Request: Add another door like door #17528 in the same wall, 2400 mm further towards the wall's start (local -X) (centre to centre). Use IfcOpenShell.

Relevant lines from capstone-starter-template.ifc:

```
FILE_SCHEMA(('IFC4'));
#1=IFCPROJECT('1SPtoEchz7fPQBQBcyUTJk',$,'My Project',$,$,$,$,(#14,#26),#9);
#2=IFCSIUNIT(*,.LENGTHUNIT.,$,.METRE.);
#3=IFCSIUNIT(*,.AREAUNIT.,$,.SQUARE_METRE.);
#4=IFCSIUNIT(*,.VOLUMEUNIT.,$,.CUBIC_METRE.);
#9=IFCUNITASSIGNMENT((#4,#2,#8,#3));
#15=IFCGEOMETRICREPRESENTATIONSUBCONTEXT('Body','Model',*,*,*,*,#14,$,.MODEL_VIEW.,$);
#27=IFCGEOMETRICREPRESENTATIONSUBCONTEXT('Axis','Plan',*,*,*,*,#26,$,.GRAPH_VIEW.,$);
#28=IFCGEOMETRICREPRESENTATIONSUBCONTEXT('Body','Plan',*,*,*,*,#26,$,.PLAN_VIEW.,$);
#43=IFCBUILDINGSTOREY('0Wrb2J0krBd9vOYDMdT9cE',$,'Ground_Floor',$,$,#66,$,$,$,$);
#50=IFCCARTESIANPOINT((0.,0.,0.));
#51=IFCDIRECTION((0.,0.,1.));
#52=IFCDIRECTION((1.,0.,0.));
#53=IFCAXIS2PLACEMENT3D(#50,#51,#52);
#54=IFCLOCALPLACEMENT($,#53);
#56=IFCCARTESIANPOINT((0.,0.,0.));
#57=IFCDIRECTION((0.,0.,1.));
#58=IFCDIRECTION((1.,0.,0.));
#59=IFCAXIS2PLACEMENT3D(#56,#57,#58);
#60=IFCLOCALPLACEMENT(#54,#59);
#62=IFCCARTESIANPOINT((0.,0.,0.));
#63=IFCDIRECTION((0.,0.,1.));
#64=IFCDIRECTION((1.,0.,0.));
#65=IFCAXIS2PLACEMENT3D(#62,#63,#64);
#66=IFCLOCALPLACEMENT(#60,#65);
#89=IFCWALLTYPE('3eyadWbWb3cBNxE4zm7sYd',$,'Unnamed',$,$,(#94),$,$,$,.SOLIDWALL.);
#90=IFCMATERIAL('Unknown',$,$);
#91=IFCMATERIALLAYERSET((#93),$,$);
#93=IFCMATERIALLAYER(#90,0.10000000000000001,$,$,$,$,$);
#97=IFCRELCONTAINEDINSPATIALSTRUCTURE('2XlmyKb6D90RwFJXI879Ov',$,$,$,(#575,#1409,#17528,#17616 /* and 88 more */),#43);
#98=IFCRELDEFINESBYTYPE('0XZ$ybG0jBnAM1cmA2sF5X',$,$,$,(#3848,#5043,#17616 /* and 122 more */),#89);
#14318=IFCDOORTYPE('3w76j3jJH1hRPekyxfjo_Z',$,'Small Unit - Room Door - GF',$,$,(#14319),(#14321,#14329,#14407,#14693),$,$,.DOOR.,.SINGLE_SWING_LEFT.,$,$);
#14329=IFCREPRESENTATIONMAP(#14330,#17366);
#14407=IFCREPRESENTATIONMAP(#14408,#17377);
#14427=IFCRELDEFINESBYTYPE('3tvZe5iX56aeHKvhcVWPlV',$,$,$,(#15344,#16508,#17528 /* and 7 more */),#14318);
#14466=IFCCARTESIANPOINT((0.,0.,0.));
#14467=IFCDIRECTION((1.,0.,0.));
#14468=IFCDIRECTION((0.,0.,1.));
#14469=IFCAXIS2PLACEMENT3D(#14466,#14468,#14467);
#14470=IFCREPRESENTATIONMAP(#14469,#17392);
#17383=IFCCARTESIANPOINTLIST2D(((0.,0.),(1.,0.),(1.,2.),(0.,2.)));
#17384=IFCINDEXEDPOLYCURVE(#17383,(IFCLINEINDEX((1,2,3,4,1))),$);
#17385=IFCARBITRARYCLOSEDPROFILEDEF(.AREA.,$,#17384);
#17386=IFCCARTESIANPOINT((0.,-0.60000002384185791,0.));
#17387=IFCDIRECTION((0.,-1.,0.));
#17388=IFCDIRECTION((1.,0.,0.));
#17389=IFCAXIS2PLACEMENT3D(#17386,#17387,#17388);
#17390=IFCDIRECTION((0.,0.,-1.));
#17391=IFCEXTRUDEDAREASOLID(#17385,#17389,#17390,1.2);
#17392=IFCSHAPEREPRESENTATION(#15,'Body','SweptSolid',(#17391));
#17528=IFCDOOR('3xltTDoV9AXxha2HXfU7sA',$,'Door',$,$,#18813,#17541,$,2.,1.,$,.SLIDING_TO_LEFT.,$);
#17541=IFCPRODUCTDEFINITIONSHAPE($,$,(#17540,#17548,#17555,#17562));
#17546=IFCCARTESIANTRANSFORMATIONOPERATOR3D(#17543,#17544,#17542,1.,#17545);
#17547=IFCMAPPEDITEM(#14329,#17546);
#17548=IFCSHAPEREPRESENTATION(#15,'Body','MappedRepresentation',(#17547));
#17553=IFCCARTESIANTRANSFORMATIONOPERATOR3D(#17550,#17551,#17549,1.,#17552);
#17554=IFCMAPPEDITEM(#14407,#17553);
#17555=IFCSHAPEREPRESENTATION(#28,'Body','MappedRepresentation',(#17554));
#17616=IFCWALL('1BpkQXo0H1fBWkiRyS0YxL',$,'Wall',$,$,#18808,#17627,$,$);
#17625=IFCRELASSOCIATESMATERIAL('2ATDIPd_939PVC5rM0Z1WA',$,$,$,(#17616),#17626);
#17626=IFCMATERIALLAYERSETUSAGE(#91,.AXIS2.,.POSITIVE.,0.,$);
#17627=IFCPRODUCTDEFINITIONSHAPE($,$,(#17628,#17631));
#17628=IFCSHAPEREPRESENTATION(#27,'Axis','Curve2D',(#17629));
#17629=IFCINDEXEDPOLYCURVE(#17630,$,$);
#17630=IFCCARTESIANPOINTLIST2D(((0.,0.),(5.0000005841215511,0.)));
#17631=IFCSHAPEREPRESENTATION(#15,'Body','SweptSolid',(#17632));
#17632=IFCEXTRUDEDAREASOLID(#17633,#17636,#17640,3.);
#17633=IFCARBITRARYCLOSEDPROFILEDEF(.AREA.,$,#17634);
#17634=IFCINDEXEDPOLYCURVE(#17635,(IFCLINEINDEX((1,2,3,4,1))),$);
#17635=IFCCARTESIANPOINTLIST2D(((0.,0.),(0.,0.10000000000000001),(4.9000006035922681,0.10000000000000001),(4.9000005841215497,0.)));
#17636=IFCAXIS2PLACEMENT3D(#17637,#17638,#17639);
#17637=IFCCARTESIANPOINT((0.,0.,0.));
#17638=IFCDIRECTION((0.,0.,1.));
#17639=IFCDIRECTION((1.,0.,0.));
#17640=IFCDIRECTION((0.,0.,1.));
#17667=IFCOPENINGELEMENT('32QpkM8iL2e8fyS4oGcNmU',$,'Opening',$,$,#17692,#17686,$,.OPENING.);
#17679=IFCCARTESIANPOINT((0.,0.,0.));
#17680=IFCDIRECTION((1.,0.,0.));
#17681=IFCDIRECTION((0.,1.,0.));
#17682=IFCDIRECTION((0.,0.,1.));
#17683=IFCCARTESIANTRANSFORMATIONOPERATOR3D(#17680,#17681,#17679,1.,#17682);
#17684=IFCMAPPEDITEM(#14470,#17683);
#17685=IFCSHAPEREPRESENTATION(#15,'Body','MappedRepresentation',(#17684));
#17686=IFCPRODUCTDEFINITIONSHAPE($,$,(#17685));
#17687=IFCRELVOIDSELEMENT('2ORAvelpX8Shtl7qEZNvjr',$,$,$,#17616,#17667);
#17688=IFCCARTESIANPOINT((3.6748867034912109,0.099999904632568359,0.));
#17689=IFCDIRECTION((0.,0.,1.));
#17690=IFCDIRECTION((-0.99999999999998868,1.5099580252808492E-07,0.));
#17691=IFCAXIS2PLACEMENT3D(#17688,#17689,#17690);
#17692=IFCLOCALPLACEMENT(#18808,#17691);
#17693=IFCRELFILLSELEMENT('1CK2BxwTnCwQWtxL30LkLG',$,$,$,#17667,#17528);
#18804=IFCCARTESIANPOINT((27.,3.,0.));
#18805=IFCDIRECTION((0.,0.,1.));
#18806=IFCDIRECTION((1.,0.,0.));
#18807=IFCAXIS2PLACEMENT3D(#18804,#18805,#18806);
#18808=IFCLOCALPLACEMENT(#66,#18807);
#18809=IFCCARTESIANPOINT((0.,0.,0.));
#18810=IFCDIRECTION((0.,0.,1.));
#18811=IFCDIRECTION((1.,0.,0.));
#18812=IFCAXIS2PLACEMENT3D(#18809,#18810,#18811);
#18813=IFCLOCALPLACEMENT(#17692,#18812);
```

```python
import ifcopenshell
import ifcopenshell.api.feature
import ifcopenshell.api.geometry
import ifcopenshell.api.root
import ifcopenshell.geom
import ifcopenshell.util.element
import ifcopenshell.util.placement
import ifcopenshell.util.shape

model = ifcopenshell.open("capstone-starter-template.ifc")
settings = ifcopenshell.geom.settings()


def volume(element):
    """Net volume in cubic metres, openings subtracted."""
    shape = ifcopenshell.geom.create_shape(settings, element)
    return ifcopenshell.util.shape.get_volume(shape.geometry)


door = model.by_id(17528)
opening = door.FillsVoids[0].RelatingOpeningElement
wall = opening.VoidsElements[0].RelatingBuildingElement
before = volume(wall)
shift = ifcopenshell.util.placement.get_local_placement(wall.ObjectPlacement)[:3, 0] * -2.4

# copy_class copies the void relationship, type, container and properties, but no geometry.
new_opening = ifcopenshell.api.root.copy_class(model, product=opening)
new_opening.Representation = ifcopenshell.util.element.copy_deep(
    model, opening.Representation, exclude=["IfcGeometricRepresentationContext", "IfcRepresentationMap"]
)
new_door = ifcopenshell.api.root.copy_class(model, product=door)
new_door.Representation = ifcopenshell.util.element.copy_deep(
    model, door.Representation, exclude=["IfcGeometricRepresentationContext", "IfcRepresentationMap"]
)
ifcopenshell.api.feature.add_filling(model, opening=new_opening, element=new_door)

for old, new in ((opening, new_opening), (door, new_door)):
    matrix = ifcopenshell.util.placement.get_local_placement(old.ObjectPlacement)
    matrix[:3, 3] += shift
    ifcopenshell.api.geometry.edit_object_placement(model, product=new, matrix=matrix, is_si=False)

after = volume(wall)

print(f"wall volume {before:.3f} -> {after:.3f} m3")

model.write("capstone-starter-template_rev.ifc")
```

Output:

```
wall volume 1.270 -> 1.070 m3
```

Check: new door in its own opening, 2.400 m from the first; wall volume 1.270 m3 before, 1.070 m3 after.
